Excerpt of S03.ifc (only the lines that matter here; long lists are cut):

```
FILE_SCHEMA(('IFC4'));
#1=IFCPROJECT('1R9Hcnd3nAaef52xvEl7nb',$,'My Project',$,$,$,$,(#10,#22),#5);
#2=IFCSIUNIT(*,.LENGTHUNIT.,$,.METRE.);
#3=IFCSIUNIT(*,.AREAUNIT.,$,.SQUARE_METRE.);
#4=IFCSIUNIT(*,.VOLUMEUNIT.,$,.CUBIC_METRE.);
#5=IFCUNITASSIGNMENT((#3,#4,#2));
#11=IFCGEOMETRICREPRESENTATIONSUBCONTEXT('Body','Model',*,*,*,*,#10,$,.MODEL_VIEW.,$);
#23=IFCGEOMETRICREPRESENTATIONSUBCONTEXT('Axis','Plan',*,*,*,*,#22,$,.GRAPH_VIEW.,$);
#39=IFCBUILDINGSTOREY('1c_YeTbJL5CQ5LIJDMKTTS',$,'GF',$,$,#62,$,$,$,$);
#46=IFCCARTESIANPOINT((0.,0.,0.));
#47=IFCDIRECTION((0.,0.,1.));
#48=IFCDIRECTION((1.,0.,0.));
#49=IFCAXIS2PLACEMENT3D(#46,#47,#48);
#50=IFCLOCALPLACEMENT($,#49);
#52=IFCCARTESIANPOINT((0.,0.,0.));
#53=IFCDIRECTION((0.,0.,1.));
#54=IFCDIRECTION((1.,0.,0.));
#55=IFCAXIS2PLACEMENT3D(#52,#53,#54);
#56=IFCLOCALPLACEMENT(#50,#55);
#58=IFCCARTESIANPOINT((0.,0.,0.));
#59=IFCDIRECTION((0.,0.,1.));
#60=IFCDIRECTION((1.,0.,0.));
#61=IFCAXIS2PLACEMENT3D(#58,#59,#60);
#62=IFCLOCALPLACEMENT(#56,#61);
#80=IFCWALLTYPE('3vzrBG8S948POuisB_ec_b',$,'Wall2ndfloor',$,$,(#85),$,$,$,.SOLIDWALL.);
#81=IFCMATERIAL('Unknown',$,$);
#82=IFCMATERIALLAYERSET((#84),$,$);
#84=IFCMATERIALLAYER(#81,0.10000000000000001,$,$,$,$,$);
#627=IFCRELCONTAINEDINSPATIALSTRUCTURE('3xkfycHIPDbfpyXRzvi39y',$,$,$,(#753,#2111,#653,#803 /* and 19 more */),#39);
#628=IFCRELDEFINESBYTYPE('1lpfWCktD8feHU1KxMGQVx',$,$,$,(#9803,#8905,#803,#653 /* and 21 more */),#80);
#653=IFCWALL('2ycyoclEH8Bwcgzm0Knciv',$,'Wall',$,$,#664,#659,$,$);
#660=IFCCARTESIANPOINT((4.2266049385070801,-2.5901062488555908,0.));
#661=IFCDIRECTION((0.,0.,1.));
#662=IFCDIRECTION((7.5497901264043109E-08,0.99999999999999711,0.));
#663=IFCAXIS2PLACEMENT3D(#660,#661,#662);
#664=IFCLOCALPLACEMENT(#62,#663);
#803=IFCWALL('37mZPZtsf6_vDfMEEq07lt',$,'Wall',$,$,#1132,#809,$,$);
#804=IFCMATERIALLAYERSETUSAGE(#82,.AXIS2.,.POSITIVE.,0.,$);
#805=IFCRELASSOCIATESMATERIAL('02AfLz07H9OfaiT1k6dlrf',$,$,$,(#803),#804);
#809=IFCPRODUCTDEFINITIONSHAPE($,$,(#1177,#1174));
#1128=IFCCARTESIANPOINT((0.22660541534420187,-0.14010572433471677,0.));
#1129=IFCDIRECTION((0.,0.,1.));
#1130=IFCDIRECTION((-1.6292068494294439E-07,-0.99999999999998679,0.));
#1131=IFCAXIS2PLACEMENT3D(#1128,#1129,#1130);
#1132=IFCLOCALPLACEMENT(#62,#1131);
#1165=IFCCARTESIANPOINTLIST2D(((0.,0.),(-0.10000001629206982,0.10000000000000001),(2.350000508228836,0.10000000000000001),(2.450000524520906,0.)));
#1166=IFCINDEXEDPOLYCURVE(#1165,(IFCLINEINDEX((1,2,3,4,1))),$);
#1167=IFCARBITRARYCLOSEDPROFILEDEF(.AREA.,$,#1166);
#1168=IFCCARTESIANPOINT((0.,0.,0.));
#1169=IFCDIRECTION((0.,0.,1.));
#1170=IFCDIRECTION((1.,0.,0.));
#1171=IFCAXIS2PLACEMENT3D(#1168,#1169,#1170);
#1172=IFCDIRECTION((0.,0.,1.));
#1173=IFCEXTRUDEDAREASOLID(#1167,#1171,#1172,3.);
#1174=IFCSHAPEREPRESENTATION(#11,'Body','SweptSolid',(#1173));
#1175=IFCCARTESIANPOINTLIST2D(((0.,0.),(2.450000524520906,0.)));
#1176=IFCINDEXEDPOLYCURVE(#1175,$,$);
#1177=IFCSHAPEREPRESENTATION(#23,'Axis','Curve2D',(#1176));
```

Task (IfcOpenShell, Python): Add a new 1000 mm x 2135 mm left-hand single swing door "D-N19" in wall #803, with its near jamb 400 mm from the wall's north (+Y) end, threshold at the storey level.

```python
import numpy as np
import ifcopenshell
import ifcopenshell.api.feature
import ifcopenshell.api.geometry
import ifcopenshell.api.root
import ifcopenshell.api.spatial
import ifcopenshell.geom
import ifcopenshell.util.element
import ifcopenshell.util.placement
import ifcopenshell.util.representation
import ifcopenshell.util.shape
import ifcopenshell.util.unit

model = ifcopenshell.open("S03.ifc")
unit_scale = ifcopenshell.util.unit.calculate_unit_scale(model)
settings = ifcopenshell.geom.settings()


def volume(element):
    """Net volume in cubic metres, openings subtracted."""
    shape = ifcopenshell.geom.create_shape(settings, element)
    return ifcopenshell.util.shape.get_volume(shape.geometry)


wall = model.by_id(803)
storey = ifcopenshell.util.element.get_container(wall, ifc_class="IfcBuildingStorey")
context = ifcopenshell.util.representation.get_context(model, "Model", "Body", "MODEL_VIEW")
before = volume(wall)

width, height, from_end, sill = 1, 2.135, 0.4, 0.0  # metres

# The wall runs along its own X axis, and the end named is its -X end.
wall_shape = ifcopenshell.geom.create_shape(settings, wall)
x, y, z = ifcopenshell.util.shape.get_vertices(wall_shape.geometry).T
start = x.min() + from_end
face, thickness = float(y.min()), float(y.max() - y.min())
wall_matrix = ifcopenshell.util.placement.get_local_placement(wall.ObjectPlacement)
level = ifcopenshell.util.placement.get_local_placement(storey.ObjectPlacement)[2, 3]


def in_wall(x, y):
    """Placement at x, y metres in the wall's axes, at sill height."""
    matrix = wall_matrix.copy()
    matrix[:, 3] = wall_matrix @ np.array([x / unit_scale, y / unit_scale, 0.0, 1.0])
    matrix[2, 3] = level + sill / unit_scale
    return matrix


# Opening: a box that overshoots both wall faces by 50 mm.
opening = ifcopenshell.api.root.create_entity(model, ifc_class="IfcOpeningElement", predefined_type="OPENING")
box = ifcopenshell.api.geometry.add_wall_representation(
    model, context=context, length=width, height=height, thickness=thickness + 0.1
)
ifcopenshell.api.geometry.assign_representation(model, product=opening, representation=box)
ifcopenshell.api.geometry.edit_object_placement(model, product=opening, matrix=in_wall(start, face - 0.05), is_si=False)
ifcopenshell.api.feature.add_feature(model, feature=opening, element=wall)

door = ifcopenshell.api.root.create_entity(model, ifc_class="IfcDoor", name="D-N19", predefined_type="DOOR")
door.OverallWidth, door.OverallHeight = width / unit_scale, height / unit_scale
door.OperationType = "SINGLE_SWING_LEFT"
body = ifcopenshell.api.geometry.add_door_representation(
    model,
    context=context,
    overall_width=door.OverallWidth,
    overall_height=door.OverallHeight,
    operation_type="SINGLE_SWING_LEFT",
    lining_properties={"LiningDepth": thickness / unit_scale, "ThresholdDepth": thickness / unit_scale},
)
ifcopenshell.api.geometry.assign_representation(model, product=door, representation=body)
ifcopenshell.api.spatial.assign_container(model, products=[door], relating_structure=storey)
ifcopenshell.api.feature.add_filling(model, opening=opening, element=door)

# The lining spans the wall, so the door starts at the wall face.
ifcopenshell.api.geometry.edit_object_placement(model, product=door, matrix=in_wall(start, face), is_si=False)

after = volume(wall)

print(f"wall volume {before:.3f} -> {after:.3f} m3")

model.write("S03_updated.ifc")
```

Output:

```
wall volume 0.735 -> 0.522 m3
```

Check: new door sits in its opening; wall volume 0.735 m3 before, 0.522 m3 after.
